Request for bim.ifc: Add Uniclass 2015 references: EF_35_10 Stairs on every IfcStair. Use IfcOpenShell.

First a look at what the model holds.

```python
import ifcopenshell

model = ifcopenshell.open("bim.ifc")
print(model.schema)
print("classifications:", [c.Name for c in model.by_type("IfcClassification")])
for ifc_class in ("IfcDoor", "IfcRoof", "IfcStair", "IfcWall", "IfcWindow"):
    print(ifc_class, len(model.by_type(ifc_class)))
```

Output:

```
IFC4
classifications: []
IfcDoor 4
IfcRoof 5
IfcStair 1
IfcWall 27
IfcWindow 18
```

```python
import ifcopenshell
import ifcopenshell.api.classification

model = ifcopenshell.open("bim.ifc")

system = ifcopenshell.api.classification.add_classification(model, classification="Uniclass 2015")

codes = {
    "IfcStair": ("EF_35_10", "Stairs"),
}
for ifc_class, (code, name) in codes.items():
    products = model.by_type(ifc_class)
    ifcopenshell.api.classification.add_reference(
        model, products=products, classification=system, identification=code, name=name
    )
    print(code, len(products))

model.write("bim-out.ifc")
```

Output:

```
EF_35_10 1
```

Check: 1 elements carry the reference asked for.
